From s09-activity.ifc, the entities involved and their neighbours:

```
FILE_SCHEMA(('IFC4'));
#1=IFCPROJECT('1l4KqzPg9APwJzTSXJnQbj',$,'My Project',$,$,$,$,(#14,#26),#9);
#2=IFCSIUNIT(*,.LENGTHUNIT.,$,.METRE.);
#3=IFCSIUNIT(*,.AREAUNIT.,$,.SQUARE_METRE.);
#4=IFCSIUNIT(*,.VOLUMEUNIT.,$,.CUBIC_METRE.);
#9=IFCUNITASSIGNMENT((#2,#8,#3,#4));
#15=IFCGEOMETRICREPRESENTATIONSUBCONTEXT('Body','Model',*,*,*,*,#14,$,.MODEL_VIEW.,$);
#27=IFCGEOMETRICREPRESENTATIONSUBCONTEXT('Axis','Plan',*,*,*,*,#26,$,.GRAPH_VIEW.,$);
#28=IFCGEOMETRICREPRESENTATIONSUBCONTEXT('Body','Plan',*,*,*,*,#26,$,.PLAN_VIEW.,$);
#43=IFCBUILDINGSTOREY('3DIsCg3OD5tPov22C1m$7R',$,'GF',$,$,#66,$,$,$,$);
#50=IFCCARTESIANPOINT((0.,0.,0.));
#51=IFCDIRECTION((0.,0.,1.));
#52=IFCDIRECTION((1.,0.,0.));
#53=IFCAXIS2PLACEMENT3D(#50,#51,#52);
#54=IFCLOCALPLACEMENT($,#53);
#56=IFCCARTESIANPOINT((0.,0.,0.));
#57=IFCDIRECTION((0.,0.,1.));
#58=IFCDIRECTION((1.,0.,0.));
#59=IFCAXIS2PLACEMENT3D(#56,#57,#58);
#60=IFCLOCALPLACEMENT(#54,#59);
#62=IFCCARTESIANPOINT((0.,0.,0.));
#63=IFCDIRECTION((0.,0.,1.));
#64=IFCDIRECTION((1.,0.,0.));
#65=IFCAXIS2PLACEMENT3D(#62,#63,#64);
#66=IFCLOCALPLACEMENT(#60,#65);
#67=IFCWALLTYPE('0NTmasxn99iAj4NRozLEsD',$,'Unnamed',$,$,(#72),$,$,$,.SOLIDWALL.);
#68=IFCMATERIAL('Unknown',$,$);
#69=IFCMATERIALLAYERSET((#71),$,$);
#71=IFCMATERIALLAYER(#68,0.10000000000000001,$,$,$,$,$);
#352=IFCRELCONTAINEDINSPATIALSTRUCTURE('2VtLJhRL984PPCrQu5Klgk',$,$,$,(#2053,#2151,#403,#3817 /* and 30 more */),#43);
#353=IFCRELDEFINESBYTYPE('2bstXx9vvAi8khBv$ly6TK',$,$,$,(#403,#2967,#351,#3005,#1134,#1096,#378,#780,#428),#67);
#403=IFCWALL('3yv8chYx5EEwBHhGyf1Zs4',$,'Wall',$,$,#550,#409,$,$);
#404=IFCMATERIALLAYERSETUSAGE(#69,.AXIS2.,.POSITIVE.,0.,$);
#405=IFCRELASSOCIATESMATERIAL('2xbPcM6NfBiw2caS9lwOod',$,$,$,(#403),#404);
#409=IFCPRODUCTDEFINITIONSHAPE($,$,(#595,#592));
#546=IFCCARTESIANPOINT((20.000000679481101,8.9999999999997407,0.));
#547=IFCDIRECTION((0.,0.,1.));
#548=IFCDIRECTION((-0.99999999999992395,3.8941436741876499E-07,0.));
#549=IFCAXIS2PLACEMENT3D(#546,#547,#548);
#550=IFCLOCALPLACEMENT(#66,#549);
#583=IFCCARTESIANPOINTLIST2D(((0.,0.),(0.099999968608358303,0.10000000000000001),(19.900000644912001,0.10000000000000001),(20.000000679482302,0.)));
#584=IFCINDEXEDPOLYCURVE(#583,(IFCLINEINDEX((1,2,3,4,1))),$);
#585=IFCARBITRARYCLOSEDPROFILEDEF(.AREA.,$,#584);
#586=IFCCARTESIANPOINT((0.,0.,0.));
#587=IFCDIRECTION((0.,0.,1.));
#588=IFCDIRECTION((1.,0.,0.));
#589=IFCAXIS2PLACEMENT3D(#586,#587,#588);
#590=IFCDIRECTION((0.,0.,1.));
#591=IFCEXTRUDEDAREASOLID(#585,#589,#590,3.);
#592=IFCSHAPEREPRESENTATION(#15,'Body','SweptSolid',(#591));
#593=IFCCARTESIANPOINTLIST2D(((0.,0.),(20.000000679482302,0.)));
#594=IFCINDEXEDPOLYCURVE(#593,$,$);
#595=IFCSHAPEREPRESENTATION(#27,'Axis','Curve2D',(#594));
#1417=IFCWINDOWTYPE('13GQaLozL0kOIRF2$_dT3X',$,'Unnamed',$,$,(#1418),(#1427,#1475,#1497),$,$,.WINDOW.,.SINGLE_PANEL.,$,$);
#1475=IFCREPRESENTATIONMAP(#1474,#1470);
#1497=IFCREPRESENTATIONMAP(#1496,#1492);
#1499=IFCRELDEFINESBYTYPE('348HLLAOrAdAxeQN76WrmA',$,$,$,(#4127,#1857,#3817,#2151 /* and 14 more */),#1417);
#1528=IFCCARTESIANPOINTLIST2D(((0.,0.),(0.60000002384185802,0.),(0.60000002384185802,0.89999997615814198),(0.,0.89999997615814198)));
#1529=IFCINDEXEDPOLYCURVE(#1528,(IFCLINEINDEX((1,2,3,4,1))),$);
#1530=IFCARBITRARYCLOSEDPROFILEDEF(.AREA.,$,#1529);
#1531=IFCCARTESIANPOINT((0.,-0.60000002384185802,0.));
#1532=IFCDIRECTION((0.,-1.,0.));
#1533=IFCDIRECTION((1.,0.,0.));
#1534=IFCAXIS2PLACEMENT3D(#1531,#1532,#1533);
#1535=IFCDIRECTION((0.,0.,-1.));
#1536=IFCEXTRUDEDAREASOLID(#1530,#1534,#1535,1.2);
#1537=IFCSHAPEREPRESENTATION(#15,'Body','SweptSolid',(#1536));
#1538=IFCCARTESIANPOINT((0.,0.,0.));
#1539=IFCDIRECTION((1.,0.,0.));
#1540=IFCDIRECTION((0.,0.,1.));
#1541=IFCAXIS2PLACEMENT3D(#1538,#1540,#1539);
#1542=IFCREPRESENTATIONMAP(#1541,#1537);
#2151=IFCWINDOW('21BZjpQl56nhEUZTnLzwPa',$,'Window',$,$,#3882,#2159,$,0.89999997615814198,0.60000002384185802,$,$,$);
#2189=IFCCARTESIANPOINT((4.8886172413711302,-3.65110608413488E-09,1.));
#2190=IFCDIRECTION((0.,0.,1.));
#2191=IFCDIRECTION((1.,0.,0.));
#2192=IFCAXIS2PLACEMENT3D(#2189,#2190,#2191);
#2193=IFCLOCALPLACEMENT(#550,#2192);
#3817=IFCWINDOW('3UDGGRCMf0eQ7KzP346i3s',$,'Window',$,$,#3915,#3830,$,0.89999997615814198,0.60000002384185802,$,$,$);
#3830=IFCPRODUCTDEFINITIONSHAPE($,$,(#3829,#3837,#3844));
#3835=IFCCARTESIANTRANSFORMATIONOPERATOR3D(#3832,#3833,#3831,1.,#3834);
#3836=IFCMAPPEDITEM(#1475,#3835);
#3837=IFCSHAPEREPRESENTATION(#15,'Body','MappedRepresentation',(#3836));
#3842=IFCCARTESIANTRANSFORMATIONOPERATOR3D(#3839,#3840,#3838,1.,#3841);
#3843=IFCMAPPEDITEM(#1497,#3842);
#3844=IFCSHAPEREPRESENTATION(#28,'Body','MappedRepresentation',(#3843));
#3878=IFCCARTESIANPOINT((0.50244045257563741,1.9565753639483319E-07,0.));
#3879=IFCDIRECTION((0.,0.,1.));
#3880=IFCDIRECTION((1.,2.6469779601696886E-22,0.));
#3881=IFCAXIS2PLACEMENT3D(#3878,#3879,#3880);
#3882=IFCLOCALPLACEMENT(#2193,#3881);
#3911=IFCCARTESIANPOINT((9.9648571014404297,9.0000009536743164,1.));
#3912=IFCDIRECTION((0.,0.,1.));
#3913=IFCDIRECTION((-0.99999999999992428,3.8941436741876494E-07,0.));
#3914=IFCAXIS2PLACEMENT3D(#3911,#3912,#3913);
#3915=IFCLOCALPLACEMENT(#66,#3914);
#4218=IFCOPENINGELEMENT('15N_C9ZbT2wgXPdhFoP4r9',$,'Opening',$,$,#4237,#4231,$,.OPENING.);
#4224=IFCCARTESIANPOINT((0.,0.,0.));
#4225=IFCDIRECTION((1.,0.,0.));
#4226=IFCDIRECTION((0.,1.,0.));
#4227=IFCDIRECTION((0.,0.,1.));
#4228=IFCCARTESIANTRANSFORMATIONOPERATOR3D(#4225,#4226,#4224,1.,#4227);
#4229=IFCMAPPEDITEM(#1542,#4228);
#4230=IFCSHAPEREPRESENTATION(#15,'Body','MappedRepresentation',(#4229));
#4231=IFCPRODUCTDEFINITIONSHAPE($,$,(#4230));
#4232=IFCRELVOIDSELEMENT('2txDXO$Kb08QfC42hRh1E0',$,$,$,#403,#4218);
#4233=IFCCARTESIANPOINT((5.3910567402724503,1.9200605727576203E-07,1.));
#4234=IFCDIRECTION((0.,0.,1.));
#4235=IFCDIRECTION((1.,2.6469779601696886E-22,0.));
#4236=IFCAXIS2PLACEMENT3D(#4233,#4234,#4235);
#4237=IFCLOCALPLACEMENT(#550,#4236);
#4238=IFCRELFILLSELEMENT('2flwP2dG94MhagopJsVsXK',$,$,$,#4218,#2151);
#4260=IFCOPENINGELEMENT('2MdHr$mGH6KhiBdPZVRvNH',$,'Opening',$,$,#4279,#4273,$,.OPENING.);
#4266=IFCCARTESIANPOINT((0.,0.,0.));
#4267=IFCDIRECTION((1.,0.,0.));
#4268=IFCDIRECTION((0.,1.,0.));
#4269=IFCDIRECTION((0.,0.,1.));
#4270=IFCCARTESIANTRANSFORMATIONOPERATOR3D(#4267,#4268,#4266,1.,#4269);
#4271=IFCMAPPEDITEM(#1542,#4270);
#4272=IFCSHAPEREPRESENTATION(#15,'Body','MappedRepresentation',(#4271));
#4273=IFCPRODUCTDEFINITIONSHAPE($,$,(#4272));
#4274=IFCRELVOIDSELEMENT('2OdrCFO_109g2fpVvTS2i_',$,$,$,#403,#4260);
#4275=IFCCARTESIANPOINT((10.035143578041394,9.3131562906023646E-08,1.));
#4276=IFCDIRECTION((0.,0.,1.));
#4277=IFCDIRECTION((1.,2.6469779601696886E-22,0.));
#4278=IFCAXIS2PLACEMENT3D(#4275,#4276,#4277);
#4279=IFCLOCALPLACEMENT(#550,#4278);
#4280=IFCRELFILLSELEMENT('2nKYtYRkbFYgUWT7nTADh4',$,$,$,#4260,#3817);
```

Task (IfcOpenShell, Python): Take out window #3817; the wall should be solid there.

```python
import ifcopenshell
import ifcopenshell.api.feature
import ifcopenshell.api.root
import ifcopenshell.geom
import ifcopenshell.util.shape

model = ifcopenshell.open("s09-activity.ifc")
settings = ifcopenshell.geom.settings()


def volume(element):
    """Net volume in cubic metres, openings subtracted."""
    shape = ifcopenshell.geom.create_shape(settings, element)
    return ifcopenshell.util.shape.get_volume(shape.geometry)


window = model.by_id(3817)
opening = window.FillsVoids[0].RelatingOpeningElement
wall = opening.VoidsElements[0].RelatingBuildingElement
before = volume(wall)

ifcopenshell.api.root.remove_product(model, product=window)
ifcopenshell.api.feature.remove_feature(model, feature=opening)

after = volume(wall)

print(f"wall volume {before:.3f} -> {after:.3f} m3")

model.write("s09-activity_updated.ifc")
```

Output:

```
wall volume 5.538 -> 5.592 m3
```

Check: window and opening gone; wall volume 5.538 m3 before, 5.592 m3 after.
